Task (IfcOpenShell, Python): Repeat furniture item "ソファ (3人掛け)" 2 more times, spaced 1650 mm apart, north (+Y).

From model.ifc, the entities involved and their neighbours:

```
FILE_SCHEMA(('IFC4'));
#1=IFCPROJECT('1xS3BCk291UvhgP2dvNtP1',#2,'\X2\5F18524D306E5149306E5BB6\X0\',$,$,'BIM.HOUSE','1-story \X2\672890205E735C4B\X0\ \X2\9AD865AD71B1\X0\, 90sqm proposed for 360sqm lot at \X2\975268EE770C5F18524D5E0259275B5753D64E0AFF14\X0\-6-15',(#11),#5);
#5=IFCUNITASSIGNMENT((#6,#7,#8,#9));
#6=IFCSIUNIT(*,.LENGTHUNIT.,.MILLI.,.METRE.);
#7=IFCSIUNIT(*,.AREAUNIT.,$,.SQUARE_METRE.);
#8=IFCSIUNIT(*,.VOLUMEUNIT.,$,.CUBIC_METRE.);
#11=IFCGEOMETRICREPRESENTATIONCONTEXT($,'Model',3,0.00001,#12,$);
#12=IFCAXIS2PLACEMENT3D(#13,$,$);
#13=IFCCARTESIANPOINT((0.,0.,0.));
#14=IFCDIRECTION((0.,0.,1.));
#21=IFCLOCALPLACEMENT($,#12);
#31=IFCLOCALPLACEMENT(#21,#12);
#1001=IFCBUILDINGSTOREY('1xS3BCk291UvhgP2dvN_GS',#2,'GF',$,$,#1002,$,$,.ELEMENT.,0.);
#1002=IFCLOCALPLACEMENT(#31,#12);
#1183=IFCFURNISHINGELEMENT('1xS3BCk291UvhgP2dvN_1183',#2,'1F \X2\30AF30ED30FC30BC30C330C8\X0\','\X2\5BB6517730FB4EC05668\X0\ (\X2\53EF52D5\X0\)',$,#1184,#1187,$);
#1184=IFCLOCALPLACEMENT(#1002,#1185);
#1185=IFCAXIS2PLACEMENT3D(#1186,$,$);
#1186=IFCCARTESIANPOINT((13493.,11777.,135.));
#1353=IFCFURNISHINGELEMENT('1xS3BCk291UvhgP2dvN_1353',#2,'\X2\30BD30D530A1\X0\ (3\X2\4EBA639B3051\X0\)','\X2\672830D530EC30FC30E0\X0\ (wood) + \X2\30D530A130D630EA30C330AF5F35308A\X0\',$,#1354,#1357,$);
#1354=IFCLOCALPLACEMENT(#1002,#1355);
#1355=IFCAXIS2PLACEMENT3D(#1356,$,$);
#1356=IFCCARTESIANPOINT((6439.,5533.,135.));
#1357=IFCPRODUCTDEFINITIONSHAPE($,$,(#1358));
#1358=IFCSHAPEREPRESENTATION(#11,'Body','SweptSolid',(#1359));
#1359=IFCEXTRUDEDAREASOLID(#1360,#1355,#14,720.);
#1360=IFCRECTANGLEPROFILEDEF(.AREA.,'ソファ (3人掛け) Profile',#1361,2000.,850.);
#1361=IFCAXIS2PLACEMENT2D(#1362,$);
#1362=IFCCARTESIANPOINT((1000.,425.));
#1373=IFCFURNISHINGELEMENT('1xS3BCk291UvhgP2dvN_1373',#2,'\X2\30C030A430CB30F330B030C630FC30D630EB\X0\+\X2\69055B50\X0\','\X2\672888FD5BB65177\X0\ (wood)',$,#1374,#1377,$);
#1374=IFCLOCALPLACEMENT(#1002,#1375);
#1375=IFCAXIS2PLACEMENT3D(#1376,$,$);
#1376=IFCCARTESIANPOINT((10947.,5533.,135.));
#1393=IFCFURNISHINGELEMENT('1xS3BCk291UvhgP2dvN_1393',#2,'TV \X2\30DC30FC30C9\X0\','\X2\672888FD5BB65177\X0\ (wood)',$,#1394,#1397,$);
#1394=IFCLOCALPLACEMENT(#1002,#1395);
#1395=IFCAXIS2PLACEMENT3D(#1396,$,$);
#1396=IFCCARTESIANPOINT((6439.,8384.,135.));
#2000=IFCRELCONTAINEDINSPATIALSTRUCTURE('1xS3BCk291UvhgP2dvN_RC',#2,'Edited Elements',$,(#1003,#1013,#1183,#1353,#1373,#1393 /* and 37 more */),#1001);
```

```python
import numpy as np
import ifcopenshell
import ifcopenshell.api.geometry
import ifcopenshell.api.root
import ifcopenshell.util.element
import ifcopenshell.util.placement

model = ifcopenshell.open("model.ifc")


def reuse_history(source, copy):
    """copy_class also copies each property set's owner history, people and application; keep the originals."""
    for rel in copy.IsDefinedBy:
        if rel.is_a("IfcRelDefinesByProperties") and (history := rel.RelatingPropertyDefinition.OwnerHistory):
            rel.RelatingPropertyDefinition.OwnerHistory = source.OwnerHistory
            ifcopenshell.util.element.remove_deep2(model, history)


source = model.by_id(1353)
base = ifcopenshell.util.placement.get_local_placement(source.ObjectPlacement)
step = np.array([0.0, 1.0, 0.0]) * 1650.0

for i in range(1, 3):
    copy = ifcopenshell.api.root.copy_class(model, product=source)
    copy.Representation = ifcopenshell.util.element.copy_deep(
        model, source.Representation, exclude=["IfcGeometricRepresentationContext", "IfcRepresentationMap"]
    )
    reuse_history(source, copy)
    matrix = base.copy()
    matrix[:3, 3] += i * step
    print("added at", matrix[:3, 3].round(3) + 0.0)
    ifcopenshell.api.geometry.edit_object_placement(model, product=copy, matrix=matrix, is_si=False)

model.write("model_rev.ifc")
```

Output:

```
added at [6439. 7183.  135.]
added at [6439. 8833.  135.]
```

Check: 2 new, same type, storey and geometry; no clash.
